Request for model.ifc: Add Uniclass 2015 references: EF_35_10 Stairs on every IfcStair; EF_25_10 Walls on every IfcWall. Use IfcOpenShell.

First a look at what the model holds.

```python
import ifcopenshell

model = ifcopenshell.open("model.ifc")
print(model.schema)
print("classifications:", [c.Name for c in model.by_type("IfcClassification")])
for ifc_class in ("IfcDoor", "IfcRoof", "IfcStair", "IfcWall", "IfcWindow"):
    print(ifc_class, len(model.by_type(ifc_class)))
```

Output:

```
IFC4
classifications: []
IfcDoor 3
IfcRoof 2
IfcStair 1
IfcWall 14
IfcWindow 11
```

```python
import ifcopenshell
import ifcopenshell.api.classification

model = ifcopenshell.open("model.ifc")

system = ifcopenshell.api.classification.add_classification(model, classification="Uniclass 2015")

codes = {
    "IfcStair": ("EF_35_10", "Stairs"),
    "IfcWall": ("EF_25_10", "Walls"),
}
for ifc_class, (code, name) in codes.items():
    products = model.by_type(ifc_class)
    ifcopenshell.api.classification.add_reference(
        model, products=products, classification=system, identification=code, name=name
    )
    print(code, len(products))

model.write("model_updated.ifc")
```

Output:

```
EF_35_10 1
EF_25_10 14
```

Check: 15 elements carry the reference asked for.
